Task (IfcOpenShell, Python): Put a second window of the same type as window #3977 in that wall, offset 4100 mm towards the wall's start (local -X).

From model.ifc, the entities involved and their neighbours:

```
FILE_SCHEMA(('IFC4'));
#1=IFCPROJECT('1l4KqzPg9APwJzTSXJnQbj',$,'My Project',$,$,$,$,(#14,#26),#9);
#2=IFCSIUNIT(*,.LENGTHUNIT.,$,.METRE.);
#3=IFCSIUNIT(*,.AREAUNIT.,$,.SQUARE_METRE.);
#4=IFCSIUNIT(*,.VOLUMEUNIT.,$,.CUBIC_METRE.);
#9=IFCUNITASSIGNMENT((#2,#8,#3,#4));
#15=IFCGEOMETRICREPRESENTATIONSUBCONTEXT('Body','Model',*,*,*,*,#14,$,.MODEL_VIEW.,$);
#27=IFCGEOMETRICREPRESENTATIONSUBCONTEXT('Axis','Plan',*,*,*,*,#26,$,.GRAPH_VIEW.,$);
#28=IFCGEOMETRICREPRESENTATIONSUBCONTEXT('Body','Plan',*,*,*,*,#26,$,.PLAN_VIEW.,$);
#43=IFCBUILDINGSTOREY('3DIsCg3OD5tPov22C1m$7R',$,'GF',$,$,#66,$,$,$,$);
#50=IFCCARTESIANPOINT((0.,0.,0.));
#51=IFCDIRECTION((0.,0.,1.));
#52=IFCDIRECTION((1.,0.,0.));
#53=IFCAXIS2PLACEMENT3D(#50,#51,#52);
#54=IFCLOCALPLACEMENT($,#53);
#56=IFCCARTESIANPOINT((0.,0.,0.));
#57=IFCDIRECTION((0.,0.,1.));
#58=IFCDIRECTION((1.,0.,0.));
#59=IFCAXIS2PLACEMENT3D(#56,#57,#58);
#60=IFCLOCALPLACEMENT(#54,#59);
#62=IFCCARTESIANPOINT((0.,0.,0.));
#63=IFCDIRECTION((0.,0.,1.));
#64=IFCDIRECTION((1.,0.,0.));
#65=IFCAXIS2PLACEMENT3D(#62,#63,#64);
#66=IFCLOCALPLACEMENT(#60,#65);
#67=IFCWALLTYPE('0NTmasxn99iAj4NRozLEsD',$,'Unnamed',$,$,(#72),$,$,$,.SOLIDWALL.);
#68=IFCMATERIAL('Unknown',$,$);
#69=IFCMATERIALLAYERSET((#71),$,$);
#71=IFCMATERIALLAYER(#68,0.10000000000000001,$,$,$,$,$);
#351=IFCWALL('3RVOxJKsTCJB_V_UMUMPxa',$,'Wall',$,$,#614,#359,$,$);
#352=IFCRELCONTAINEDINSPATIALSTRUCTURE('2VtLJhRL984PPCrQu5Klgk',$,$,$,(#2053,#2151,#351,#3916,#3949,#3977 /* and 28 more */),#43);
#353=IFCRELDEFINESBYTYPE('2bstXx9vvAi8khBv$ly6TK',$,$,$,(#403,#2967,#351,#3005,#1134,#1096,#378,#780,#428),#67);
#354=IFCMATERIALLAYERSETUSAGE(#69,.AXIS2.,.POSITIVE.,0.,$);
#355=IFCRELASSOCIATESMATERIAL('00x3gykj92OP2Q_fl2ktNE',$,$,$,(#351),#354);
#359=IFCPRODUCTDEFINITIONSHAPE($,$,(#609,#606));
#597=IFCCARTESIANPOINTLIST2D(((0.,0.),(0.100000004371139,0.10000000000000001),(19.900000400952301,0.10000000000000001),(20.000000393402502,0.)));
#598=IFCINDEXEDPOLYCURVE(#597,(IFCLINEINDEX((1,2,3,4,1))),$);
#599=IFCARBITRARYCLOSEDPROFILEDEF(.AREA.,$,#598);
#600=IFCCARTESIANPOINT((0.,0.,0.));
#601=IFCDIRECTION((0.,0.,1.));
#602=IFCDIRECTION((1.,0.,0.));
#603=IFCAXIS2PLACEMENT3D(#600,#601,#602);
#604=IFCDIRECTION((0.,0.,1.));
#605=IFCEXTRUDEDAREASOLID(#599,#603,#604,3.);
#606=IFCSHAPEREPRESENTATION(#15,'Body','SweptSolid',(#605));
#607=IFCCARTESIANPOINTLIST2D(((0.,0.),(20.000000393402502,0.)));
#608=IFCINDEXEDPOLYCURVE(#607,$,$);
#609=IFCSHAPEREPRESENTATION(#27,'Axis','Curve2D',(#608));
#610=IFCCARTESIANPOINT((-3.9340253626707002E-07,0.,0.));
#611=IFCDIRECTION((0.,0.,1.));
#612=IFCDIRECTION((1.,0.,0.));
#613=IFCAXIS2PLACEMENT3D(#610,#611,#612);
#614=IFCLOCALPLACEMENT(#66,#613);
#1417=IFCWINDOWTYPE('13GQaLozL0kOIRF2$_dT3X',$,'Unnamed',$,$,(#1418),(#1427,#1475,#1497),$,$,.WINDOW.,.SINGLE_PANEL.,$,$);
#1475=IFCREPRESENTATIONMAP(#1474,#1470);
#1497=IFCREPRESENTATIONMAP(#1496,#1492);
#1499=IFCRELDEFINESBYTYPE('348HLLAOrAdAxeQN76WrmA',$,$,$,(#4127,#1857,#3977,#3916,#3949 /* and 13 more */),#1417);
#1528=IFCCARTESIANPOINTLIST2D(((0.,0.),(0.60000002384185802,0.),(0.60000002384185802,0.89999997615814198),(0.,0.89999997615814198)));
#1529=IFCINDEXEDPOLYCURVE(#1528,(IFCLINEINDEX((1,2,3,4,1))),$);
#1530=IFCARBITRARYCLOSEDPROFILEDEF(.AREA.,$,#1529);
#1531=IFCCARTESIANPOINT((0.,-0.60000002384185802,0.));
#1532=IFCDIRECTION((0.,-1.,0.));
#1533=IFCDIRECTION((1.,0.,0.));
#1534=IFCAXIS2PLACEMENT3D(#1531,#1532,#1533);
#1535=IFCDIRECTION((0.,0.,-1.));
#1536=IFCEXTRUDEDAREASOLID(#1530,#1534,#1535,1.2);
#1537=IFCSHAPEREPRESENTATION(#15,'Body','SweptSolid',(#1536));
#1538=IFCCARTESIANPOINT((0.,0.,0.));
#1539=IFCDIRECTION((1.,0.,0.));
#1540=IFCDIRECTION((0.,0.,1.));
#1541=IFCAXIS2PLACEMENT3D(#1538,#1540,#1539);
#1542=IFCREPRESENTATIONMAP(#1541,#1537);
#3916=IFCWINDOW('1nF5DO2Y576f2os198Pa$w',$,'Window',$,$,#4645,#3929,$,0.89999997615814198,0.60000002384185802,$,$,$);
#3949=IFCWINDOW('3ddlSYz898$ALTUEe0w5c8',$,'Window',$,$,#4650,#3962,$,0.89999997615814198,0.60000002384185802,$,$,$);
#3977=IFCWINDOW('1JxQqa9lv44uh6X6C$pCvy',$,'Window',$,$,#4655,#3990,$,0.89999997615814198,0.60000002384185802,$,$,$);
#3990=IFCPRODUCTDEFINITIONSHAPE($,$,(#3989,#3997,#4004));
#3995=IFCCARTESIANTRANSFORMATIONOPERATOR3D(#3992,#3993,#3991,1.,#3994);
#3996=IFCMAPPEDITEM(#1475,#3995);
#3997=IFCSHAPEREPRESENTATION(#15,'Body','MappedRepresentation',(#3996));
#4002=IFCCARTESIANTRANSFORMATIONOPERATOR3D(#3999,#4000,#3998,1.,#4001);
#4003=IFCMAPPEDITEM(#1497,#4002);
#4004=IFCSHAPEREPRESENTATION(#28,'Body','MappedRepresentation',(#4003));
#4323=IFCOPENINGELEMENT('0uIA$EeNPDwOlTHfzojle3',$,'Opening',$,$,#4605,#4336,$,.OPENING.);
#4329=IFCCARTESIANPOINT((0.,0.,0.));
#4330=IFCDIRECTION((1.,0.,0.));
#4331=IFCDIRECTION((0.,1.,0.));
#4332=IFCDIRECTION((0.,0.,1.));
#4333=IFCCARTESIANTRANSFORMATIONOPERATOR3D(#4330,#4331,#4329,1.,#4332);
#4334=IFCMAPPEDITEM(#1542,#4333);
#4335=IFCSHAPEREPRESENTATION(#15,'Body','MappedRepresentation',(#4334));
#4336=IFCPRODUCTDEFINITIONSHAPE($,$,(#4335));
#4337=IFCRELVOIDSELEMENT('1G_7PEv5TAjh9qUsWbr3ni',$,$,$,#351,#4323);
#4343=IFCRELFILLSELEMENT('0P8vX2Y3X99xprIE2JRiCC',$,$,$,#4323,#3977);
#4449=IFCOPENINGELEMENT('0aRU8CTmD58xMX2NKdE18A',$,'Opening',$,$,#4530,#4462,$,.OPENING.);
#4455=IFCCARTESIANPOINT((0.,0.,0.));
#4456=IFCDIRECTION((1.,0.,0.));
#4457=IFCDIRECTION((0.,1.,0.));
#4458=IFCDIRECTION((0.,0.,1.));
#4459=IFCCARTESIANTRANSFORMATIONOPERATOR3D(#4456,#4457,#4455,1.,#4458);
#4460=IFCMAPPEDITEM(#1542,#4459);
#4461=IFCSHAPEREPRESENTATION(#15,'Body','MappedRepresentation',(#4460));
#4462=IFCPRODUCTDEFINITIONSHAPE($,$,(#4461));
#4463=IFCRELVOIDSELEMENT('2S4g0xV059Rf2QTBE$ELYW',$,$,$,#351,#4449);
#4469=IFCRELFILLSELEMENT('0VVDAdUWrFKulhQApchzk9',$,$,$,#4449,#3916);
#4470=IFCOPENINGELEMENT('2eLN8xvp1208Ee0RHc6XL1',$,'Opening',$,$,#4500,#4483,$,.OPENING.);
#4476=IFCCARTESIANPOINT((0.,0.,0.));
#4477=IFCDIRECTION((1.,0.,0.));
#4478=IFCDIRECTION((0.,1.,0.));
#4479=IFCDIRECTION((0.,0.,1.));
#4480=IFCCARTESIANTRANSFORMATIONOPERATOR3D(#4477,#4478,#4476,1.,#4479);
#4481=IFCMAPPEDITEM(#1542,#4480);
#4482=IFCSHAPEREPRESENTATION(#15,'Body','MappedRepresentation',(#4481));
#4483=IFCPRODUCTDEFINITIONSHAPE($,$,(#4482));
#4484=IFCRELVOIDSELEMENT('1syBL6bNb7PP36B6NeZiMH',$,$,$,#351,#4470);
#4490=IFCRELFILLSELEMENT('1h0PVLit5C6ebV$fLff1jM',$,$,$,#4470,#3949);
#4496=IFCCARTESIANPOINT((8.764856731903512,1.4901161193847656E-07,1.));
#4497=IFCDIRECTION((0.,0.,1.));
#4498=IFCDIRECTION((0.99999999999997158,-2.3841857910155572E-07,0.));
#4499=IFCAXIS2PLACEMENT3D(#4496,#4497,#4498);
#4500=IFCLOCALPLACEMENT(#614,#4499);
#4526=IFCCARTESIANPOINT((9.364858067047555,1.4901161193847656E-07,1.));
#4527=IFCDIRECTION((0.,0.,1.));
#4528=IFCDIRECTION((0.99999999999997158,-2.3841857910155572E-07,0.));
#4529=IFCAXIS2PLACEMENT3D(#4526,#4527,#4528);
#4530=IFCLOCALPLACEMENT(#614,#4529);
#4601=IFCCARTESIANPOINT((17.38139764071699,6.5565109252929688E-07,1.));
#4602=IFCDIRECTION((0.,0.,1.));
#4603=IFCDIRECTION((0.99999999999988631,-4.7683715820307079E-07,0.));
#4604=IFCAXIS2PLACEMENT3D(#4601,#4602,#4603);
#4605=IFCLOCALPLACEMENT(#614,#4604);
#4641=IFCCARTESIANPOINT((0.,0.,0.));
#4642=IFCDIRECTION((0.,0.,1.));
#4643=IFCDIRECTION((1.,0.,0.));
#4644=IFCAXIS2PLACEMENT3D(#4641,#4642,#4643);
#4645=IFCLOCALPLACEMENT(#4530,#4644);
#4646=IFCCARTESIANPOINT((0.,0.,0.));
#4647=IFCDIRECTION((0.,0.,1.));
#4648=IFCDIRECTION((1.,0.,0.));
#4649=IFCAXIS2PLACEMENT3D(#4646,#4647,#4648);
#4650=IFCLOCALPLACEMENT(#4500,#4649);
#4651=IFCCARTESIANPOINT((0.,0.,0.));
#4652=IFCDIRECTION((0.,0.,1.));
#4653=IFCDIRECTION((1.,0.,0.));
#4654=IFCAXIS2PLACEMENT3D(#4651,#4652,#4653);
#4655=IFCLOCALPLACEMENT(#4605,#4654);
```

```python
import ifcopenshell
import ifcopenshell.api.feature
import ifcopenshell.api.geometry
import ifcopenshell.api.root
import ifcopenshell.geom
import ifcopenshell.util.element
import ifcopenshell.util.placement
import ifcopenshell.util.shape
import ifcopenshell.util.unit

model = ifcopenshell.open("model.ifc")
unit_scale = ifcopenshell.util.unit.calculate_unit_scale(model)
settings = ifcopenshell.geom.settings()


def volume(element):
    """Net volume in cubic metres, openings subtracted."""
    shape = ifcopenshell.geom.create_shape(settings, element)
    return ifcopenshell.util.shape.get_volume(shape.geometry)


window = model.by_guid("1JxQqa9lv44uh6X6C$pCvy")
opening = window.FillsVoids[0].RelatingOpeningElement
wall = opening.VoidsElements[0].RelatingBuildingElement
before = volume(wall)
shift = ifcopenshell.util.placement.get_local_placement(wall.ObjectPlacement)[:3, 0] * -4.1 / unit_scale

# copy_class copies the void relationship, type, container and properties, but no geometry.
new_opening = ifcopenshell.api.root.copy_class(model, product=opening)
new_opening.Representation = ifcopenshell.util.element.copy_deep(
    model, opening.Representation, exclude=["IfcGeometricRepresentationContext", "IfcRepresentationMap"]
)
new_window = ifcopenshell.api.root.copy_class(model, product=window)
new_window.Representation = ifcopenshell.util.element.copy_deep(
    model, window.Representation, exclude=["IfcGeometricRepresentationContext", "IfcRepresentationMap"]
)
ifcopenshell.api.feature.add_filling(model, opening=new_opening, element=new_window)

for old, new in ((opening, new_opening), (window, new_window)):
    matrix = ifcopenshell.util.placement.get_local_placement(old.ObjectPlacement)
    matrix[:3, 3] += shift
    ifcopenshell.api.geometry.edit_object_placement(model, product=new, matrix=matrix, is_si=False)

after = volume(wall)

print(f"wall volume {before:.3f} -> {after:.3f} m3")

model.write("model_v2.ifc")
```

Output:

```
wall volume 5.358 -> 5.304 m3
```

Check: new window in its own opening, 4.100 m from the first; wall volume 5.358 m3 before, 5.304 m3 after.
